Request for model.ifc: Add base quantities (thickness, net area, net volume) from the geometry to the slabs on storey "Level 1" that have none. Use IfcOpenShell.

First a look at what the model holds.

```python
import ifcopenshell
import ifcopenshell.util.element
import ifcopenshell.util.unit

model = ifcopenshell.open("model.ifc")
print(model.schema)
for unit_type in ("LENGTHUNIT", "AREAUNIT", "VOLUMEUNIT"):
    print(unit_type, ifcopenshell.util.unit.calculate_unit_scale(model, unit_type))
storey = next(s for s in model.by_type("IfcBuildingStorey") if s.Name == "Level 1")
slabs = [e for e in ifcopenshell.util.element.get_decomposition(storey) if e.is_a("IfcSlab")]
for e in sorted(slabs, key=lambda e: e.id()):
    print(e.id(), e.is_a(), e.Name, list(ifcopenshell.util.element.get_psets(e, qtos_only=True)), sep=" | ")
```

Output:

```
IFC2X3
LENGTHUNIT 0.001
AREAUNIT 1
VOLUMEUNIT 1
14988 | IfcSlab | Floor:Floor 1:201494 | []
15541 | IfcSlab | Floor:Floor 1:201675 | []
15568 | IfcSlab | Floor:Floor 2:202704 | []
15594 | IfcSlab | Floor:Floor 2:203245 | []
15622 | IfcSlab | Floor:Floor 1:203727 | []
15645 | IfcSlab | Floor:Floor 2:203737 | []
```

```python
import ifcopenshell
import ifcopenshell.api.pset
import ifcopenshell.geom
import ifcopenshell.util.element
import ifcopenshell.util.shape
import ifcopenshell.util.unit

model = ifcopenshell.open("model.ifc")
unit_scale = ifcopenshell.util.unit.calculate_unit_scale(model)
area_scale = ifcopenshell.util.unit.calculate_unit_scale(model, "AREAUNIT")
volume_scale = ifcopenshell.util.unit.calculate_unit_scale(model, "VOLUMEUNIT")
settings = ifcopenshell.geom.settings()

storey = next(s for s in model.by_type("IfcBuildingStorey") if s.Name == "Level 1")
slabs = [e for e in ifcopenshell.util.element.get_decomposition(storey) if e.is_a("IfcSlab")]

for e in sorted(slabs, key=lambda e: e.id()):
    if ifcopenshell.util.element.get_psets(e, qtos_only=True, should_inherit=False):
        continue
    # Geometry comes back in metres, in the element's own axes.
    shape = ifcopenshell.geom.create_shape(settings, e)
    values = {
        "Width": ifcopenshell.util.shape.get_z(shape.geometry) / unit_scale,
        "NetArea": ifcopenshell.util.shape.get_footprint_area(shape.geometry) / area_scale,
        "NetVolume": ifcopenshell.util.shape.get_volume(shape.geometry) / volume_scale,
    }
    qto = ifcopenshell.api.pset.add_qto(model, product=e, name="BaseQuantities")
    ifcopenshell.api.pset.edit_qto(model, qto=qto, properties=values)
    print(e.id(), {k: round(v, 3) for k, v in values.items()})

model.write("model_rev.ifc")
```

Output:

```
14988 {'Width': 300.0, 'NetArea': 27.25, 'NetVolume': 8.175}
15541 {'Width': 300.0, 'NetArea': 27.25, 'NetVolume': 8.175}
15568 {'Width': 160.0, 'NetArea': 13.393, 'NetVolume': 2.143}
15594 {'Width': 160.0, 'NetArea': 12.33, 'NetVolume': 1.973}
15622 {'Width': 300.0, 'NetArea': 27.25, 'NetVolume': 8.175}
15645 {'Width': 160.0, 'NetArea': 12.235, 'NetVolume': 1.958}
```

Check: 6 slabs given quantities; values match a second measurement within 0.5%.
